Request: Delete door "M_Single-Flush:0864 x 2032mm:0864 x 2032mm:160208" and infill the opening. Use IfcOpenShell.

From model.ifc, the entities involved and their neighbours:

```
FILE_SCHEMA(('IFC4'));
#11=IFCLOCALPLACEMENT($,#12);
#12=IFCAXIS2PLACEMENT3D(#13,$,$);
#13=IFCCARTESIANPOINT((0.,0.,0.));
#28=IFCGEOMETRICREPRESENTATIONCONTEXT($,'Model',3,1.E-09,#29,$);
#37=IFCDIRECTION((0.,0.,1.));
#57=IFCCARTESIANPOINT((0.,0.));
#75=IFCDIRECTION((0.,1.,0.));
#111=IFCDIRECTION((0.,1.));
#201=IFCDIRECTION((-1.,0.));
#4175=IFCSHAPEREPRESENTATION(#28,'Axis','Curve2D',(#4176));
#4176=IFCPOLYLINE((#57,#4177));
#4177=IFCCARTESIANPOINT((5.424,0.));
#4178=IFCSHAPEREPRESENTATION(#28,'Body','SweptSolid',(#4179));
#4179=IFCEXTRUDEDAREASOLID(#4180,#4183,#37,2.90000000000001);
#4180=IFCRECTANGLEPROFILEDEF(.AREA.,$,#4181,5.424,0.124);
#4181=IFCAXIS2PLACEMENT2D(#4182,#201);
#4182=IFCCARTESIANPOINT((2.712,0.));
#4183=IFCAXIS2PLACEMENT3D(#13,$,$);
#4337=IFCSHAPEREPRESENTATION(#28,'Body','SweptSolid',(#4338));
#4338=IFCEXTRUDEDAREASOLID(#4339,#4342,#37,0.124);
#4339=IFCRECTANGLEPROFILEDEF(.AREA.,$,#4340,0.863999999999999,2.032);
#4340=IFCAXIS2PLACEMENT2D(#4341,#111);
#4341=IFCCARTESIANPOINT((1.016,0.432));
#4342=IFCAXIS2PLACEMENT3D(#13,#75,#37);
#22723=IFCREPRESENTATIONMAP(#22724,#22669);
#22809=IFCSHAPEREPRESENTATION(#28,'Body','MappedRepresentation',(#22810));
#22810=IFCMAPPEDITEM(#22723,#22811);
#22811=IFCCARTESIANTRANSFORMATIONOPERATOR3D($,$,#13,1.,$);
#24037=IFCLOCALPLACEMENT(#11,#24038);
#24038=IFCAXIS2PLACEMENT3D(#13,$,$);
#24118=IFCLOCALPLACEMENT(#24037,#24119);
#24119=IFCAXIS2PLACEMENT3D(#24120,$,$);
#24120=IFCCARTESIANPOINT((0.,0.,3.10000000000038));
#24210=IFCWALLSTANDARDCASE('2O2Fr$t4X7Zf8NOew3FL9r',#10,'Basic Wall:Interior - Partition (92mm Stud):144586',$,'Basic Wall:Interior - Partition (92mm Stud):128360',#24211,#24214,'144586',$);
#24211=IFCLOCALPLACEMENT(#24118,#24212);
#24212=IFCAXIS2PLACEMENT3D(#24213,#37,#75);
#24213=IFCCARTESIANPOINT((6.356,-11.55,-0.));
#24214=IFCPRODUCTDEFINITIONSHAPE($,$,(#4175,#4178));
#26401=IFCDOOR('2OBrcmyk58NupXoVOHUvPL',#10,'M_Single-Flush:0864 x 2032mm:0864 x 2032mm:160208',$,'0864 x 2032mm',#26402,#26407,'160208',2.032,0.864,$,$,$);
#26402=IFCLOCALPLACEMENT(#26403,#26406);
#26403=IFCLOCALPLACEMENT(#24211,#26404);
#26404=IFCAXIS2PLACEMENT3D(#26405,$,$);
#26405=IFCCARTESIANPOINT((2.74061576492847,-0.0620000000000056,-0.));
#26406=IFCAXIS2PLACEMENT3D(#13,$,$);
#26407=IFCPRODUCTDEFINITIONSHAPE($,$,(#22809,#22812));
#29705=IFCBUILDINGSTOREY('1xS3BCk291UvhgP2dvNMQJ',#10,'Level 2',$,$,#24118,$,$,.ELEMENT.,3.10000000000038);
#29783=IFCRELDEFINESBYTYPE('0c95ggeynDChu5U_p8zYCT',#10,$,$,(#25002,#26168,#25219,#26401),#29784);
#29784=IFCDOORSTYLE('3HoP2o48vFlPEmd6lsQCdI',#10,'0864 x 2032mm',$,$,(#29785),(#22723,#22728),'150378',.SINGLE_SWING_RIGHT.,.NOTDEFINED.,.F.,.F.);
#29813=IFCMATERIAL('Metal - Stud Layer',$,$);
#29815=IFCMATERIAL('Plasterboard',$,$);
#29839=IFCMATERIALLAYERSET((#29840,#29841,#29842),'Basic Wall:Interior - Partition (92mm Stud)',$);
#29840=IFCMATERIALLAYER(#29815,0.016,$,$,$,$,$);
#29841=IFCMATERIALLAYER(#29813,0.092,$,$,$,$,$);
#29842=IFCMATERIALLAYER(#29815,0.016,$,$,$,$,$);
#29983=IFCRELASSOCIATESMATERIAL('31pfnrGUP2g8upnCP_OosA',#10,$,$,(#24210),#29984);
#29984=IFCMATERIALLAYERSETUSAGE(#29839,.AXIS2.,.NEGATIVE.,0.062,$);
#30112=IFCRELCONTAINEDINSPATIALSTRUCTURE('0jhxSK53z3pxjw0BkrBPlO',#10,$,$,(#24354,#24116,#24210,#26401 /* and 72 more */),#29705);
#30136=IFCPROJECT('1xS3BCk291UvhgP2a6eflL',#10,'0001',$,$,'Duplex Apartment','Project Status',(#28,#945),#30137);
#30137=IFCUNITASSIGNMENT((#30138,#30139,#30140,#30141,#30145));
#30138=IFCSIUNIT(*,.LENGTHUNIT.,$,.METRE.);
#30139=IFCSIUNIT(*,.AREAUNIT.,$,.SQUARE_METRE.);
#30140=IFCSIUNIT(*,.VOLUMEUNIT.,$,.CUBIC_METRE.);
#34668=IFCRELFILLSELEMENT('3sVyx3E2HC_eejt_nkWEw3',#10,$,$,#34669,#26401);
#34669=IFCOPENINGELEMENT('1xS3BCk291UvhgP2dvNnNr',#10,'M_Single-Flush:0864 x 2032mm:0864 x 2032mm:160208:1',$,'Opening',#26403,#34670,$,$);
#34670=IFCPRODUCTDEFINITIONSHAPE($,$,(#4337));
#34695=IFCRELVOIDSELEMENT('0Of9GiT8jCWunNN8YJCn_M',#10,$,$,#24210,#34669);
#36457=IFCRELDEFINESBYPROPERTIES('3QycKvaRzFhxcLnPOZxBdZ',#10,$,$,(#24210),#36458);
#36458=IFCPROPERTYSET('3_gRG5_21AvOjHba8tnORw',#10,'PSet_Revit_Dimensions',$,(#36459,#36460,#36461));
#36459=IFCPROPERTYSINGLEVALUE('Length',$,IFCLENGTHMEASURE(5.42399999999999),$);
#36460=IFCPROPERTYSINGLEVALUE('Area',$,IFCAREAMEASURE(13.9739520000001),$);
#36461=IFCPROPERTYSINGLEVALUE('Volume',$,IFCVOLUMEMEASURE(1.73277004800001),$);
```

```python
import ifcopenshell
import ifcopenshell.api.feature
import ifcopenshell.api.pset
import ifcopenshell.api.root
import ifcopenshell.geom
import ifcopenshell.util.element
import ifcopenshell.util.shape
import ifcopenshell.util.unit

model = ifcopenshell.open("model.ifc")
area_scale = ifcopenshell.util.unit.calculate_unit_scale(model, "AREAUNIT")
volume_scale = ifcopenshell.util.unit.calculate_unit_scale(model, "VOLUMEUNIT")
settings = ifcopenshell.geom.settings()


def volume(element):
    """Net volume in cubic metres, openings subtracted."""
    shape = ifcopenshell.geom.create_shape(settings, element)
    return ifcopenshell.util.shape.get_volume(shape.geometry)


door = model.by_guid("2OBrcmyk58NupXoVOHUvPL")
opening = door.FillsVoids[0].RelatingOpeningElement
wall = opening.VoidsElements[0].RelatingBuildingElement
before = volume(wall)

ifcopenshell.api.root.remove_product(model, product=door)
ifcopenshell.api.feature.remove_feature(model, feature=opening)

after = volume(wall)
thickness = 0.124  # wall thickness in metres

# Update the wall's stored quantities.
pset = model.by_id(ifcopenshell.util.element.get_pset(wall, "PSet_Revit_Dimensions", should_inherit=False)["id"])
ifcopenshell.api.pset.edit_pset(model, pset=pset, properties={
    "Area": model.create_entity("IfcAreaMeasure", after / thickness / area_scale),
    "Volume": model.create_entity("IfcVolumeMeasure", after / volume_scale),
})

print(f"wall volume {before:.3f} -> {after:.3f} m3")

model.write("model_rev.ifc")
```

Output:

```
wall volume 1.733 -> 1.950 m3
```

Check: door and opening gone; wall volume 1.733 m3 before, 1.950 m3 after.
